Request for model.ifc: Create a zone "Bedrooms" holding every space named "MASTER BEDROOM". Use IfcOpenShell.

First a look at what the model holds.

```python
import ifcopenshell

model = ifcopenshell.open("model.ifc")
print(model.schema)
seen = {}
for space in model.by_type("IfcSpace"):
    seen[space.LongName] = seen.get(space.LongName, 0) + 1
for name, count in sorted(seen.items(), key=str):
    print(count, "x", name)
print("zones:", [z.Name for z in model.by_type("IfcZone")][:20])
```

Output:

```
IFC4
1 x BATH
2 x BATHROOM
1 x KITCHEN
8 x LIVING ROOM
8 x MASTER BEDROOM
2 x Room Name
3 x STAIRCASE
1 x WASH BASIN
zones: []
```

```python
import ifcopenshell
import ifcopenshell.api.group
import ifcopenshell.api.root

model = ifcopenshell.open("model.ifc")

names = {"MASTER BEDROOM"}
spaces = [s for s in model.by_type("IfcSpace") if s.LongName in names]

zone = ifcopenshell.api.root.create_entity(model, ifc_class="IfcZone", name="Bedrooms")
ifcopenshell.api.group.assign_group(model, products=spaces, group=zone)
print(len(spaces), "spaces in", zone.Name)

model.write("model_v2.ifc")
```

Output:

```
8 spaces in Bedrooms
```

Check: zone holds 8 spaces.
